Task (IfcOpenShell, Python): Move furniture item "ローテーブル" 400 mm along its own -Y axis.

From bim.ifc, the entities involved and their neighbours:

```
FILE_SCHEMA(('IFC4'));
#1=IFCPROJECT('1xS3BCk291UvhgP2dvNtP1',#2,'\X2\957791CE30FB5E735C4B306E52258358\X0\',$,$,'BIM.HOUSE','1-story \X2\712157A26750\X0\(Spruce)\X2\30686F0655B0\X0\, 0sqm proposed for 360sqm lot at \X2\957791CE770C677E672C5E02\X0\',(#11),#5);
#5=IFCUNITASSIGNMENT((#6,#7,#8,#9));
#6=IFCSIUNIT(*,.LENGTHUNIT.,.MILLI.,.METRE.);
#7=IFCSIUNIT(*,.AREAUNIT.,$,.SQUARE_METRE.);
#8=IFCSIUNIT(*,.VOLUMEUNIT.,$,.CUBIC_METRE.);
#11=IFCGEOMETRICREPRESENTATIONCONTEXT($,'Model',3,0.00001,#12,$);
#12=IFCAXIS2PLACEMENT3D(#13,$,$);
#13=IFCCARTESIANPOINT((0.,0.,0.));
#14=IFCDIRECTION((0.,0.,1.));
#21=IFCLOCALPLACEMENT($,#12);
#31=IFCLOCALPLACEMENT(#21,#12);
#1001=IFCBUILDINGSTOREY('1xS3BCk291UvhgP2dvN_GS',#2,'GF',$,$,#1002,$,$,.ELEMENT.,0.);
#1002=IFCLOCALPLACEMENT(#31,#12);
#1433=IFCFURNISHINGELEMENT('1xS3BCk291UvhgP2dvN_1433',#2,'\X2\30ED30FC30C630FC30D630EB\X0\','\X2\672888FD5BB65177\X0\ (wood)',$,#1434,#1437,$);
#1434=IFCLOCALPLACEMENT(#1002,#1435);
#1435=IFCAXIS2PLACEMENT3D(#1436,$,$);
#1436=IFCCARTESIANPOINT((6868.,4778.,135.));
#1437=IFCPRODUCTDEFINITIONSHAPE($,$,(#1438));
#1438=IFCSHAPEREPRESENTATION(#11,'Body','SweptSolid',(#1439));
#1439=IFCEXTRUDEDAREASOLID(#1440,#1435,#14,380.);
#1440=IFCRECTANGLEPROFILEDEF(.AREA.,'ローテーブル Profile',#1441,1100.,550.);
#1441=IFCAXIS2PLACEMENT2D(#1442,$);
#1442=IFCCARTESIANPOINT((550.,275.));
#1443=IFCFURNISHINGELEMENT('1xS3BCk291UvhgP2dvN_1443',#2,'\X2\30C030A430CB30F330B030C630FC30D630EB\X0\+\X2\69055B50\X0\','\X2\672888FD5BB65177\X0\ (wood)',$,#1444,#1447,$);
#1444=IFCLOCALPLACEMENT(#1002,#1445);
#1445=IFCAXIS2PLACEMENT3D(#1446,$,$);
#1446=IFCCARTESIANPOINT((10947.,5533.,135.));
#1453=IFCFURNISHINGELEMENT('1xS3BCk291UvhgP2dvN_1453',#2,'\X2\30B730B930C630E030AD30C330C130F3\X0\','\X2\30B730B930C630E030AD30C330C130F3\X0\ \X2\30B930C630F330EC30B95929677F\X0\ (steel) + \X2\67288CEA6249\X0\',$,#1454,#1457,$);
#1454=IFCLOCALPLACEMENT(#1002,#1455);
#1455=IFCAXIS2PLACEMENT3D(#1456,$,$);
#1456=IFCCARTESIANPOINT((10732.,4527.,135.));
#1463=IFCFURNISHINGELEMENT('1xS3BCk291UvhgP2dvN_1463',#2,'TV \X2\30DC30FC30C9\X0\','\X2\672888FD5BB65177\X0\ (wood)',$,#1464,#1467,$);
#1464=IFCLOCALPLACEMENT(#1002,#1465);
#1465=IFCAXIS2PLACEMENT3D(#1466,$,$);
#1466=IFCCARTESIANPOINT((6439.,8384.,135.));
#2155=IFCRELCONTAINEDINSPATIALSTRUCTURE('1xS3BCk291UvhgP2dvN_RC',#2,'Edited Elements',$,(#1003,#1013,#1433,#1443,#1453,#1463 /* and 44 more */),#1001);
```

```python
import ifcopenshell
import ifcopenshell.api.geometry
import ifcopenshell.util.placement

model = ifcopenshell.open("bim.ifc")

item = model.by_guid("1xS3BCk291UvhgP2dvN_1433")
matrix = ifcopenshell.util.placement.get_local_placement(item.ObjectPlacement)
matrix[:3, 3] -= matrix[:3, 1] * 400.0
ifcopenshell.api.geometry.edit_object_placement(model, product=item, matrix=matrix, is_si=False)

print(ifcopenshell.util.placement.get_local_placement(item.ObjectPlacement).round(3) + 0.0)

model.write("bim-out.ifc")
```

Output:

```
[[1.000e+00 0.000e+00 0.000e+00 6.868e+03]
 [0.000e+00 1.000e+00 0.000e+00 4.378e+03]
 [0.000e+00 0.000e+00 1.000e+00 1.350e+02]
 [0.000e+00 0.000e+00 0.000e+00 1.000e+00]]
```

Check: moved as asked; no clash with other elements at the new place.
